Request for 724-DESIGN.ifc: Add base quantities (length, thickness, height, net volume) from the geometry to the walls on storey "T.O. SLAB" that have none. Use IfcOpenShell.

First a look at what the model holds.

```python
import ifcopenshell
import ifcopenshell.util.element
import ifcopenshell.util.unit

model = ifcopenshell.open("724-DESIGN.ifc")
print(model.schema)
for unit_type in ("LENGTHUNIT", "AREAUNIT", "VOLUMEUNIT"):
    print(unit_type, ifcopenshell.util.unit.calculate_unit_scale(model, unit_type))
storey = next(s for s in model.by_type("IfcBuildingStorey") if s.Name == "T.O. SLAB")
walls = [e for e in ifcopenshell.util.element.get_decomposition(storey) if e.is_a("IfcWall")]
for e in sorted(walls, key=lambda e: e.id()):
    print(e.id(), e.is_a(), e.Name, list(ifcopenshell.util.element.get_psets(e, qtos_only=True)), sep=" | ")
```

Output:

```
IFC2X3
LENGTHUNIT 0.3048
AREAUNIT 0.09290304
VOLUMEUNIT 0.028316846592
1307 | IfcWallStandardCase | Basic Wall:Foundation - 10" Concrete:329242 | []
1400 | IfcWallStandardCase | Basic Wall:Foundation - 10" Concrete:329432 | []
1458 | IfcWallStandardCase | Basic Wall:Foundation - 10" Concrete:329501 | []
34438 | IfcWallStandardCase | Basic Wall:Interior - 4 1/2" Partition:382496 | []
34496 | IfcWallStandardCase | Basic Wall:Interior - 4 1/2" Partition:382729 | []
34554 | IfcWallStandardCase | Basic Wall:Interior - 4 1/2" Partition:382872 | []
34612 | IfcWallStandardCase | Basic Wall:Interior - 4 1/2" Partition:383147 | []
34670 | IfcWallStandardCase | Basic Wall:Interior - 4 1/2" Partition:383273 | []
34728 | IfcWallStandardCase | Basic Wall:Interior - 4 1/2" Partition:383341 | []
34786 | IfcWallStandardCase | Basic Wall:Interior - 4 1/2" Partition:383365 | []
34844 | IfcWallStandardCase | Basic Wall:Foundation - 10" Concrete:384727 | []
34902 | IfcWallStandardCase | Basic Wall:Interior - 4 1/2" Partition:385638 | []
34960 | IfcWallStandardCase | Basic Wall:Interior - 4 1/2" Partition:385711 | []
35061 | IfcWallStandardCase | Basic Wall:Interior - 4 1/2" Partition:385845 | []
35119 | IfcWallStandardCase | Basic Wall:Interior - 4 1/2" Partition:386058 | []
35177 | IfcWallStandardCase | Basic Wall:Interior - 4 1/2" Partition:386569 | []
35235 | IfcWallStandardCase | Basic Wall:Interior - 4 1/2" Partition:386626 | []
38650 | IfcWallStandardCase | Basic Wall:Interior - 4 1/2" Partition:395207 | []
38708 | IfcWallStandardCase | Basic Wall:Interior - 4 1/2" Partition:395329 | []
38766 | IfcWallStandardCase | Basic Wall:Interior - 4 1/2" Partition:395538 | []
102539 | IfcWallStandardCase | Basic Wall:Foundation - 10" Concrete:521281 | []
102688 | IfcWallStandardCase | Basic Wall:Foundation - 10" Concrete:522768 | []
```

```python
import ifcopenshell
import ifcopenshell.api.pset
import ifcopenshell.geom
import ifcopenshell.util.element
import ifcopenshell.util.shape
import ifcopenshell.util.unit

model = ifcopenshell.open("724-DESIGN.ifc")
unit_scale = ifcopenshell.util.unit.calculate_unit_scale(model)
volume_scale = ifcopenshell.util.unit.calculate_unit_scale(model, "VOLUMEUNIT")
settings = ifcopenshell.geom.settings()

storey = next(s for s in model.by_type("IfcBuildingStorey") if s.Name == "T.O. SLAB")
walls = [e for e in ifcopenshell.util.element.get_decomposition(storey) if e.is_a("IfcWall")]

for e in sorted(walls, key=lambda e: e.id()):
    if ifcopenshell.util.element.get_psets(e, qtos_only=True, should_inherit=False):
        continue
    # Geometry comes back in metres, in the element's own axes.
    shape = ifcopenshell.geom.create_shape(settings, e)
    values = {
        "Length": ifcopenshell.util.shape.get_x(shape.geometry) / unit_scale,
        "Width": ifcopenshell.util.shape.get_y(shape.geometry) / unit_scale,
        "Height": ifcopenshell.util.shape.get_z(shape.geometry) / unit_scale,
        "NetVolume": ifcopenshell.util.shape.get_volume(shape.geometry) / volume_scale,
    }
    qto = ifcopenshell.api.pset.add_qto(model, product=e, name="BaseQuantities")
    ifcopenshell.api.pset.edit_qto(model, qto=qto, properties=values)
    print(e.id(), {k: round(v, 3) for k, v in values.items()})

model.write("724-DESIGN-out.ifc")
```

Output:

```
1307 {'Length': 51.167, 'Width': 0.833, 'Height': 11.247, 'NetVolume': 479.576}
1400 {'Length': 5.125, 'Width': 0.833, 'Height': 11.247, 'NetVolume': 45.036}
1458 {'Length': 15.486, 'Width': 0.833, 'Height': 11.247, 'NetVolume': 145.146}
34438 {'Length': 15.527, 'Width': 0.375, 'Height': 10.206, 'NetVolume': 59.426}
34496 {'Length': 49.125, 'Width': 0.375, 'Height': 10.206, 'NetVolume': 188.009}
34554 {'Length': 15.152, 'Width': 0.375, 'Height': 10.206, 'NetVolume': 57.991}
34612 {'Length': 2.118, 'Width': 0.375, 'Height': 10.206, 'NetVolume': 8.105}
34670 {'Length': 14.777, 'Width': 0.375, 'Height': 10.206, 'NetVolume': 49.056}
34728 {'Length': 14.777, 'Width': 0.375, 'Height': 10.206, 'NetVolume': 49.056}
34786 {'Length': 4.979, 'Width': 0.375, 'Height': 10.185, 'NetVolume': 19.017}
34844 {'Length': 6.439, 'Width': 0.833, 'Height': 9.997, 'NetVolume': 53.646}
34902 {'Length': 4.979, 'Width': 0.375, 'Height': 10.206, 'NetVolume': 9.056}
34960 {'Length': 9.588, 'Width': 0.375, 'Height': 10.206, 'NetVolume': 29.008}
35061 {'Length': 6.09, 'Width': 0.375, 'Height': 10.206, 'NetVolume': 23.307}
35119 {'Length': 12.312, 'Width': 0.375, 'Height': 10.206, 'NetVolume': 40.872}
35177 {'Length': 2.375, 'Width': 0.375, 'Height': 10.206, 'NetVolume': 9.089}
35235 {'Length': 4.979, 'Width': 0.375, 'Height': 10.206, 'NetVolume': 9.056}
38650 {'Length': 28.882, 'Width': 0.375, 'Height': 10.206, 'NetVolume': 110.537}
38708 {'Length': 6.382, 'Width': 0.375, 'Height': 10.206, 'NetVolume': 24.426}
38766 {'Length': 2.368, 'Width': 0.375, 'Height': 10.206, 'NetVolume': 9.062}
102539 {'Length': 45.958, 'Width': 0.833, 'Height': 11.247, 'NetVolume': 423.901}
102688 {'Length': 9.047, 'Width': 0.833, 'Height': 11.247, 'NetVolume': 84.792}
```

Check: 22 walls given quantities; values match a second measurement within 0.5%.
